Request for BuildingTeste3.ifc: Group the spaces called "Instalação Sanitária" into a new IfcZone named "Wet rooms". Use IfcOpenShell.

First a look at what the model holds.

```python
import ifcopenshell

model = ifcopenshell.open("BuildingTeste3.ifc")
print(model.schema)
seen = {}
for space in model.by_type("IfcSpace"):
    seen[space.LongName] = seen.get(space.LongName, 0) + 1
for name, count in sorted(seen.items(), key=str):
    print(count, "x", name)
print("zones:", [z.Name for z in model.by_type("IfcZone")][:20])
```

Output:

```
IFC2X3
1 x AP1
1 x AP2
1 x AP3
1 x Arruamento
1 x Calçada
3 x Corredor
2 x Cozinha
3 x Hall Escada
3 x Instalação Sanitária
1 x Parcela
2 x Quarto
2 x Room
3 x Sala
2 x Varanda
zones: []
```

```python
import ifcopenshell
import ifcopenshell.api.group
import ifcopenshell.api.root

model = ifcopenshell.open("BuildingTeste3.ifc")

names = {"Instalação Sanitária"}
spaces = [s for s in model.by_type("IfcSpace") if s.LongName in names]

zone = ifcopenshell.api.root.create_entity(model, ifc_class="IfcZone", name="Wet rooms")
ifcopenshell.api.group.assign_group(model, products=spaces, group=zone)
print(len(spaces), "spaces in", zone.Name)

model.write("BuildingTeste3_updated.ifc")
```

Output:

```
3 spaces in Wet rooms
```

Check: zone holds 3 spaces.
